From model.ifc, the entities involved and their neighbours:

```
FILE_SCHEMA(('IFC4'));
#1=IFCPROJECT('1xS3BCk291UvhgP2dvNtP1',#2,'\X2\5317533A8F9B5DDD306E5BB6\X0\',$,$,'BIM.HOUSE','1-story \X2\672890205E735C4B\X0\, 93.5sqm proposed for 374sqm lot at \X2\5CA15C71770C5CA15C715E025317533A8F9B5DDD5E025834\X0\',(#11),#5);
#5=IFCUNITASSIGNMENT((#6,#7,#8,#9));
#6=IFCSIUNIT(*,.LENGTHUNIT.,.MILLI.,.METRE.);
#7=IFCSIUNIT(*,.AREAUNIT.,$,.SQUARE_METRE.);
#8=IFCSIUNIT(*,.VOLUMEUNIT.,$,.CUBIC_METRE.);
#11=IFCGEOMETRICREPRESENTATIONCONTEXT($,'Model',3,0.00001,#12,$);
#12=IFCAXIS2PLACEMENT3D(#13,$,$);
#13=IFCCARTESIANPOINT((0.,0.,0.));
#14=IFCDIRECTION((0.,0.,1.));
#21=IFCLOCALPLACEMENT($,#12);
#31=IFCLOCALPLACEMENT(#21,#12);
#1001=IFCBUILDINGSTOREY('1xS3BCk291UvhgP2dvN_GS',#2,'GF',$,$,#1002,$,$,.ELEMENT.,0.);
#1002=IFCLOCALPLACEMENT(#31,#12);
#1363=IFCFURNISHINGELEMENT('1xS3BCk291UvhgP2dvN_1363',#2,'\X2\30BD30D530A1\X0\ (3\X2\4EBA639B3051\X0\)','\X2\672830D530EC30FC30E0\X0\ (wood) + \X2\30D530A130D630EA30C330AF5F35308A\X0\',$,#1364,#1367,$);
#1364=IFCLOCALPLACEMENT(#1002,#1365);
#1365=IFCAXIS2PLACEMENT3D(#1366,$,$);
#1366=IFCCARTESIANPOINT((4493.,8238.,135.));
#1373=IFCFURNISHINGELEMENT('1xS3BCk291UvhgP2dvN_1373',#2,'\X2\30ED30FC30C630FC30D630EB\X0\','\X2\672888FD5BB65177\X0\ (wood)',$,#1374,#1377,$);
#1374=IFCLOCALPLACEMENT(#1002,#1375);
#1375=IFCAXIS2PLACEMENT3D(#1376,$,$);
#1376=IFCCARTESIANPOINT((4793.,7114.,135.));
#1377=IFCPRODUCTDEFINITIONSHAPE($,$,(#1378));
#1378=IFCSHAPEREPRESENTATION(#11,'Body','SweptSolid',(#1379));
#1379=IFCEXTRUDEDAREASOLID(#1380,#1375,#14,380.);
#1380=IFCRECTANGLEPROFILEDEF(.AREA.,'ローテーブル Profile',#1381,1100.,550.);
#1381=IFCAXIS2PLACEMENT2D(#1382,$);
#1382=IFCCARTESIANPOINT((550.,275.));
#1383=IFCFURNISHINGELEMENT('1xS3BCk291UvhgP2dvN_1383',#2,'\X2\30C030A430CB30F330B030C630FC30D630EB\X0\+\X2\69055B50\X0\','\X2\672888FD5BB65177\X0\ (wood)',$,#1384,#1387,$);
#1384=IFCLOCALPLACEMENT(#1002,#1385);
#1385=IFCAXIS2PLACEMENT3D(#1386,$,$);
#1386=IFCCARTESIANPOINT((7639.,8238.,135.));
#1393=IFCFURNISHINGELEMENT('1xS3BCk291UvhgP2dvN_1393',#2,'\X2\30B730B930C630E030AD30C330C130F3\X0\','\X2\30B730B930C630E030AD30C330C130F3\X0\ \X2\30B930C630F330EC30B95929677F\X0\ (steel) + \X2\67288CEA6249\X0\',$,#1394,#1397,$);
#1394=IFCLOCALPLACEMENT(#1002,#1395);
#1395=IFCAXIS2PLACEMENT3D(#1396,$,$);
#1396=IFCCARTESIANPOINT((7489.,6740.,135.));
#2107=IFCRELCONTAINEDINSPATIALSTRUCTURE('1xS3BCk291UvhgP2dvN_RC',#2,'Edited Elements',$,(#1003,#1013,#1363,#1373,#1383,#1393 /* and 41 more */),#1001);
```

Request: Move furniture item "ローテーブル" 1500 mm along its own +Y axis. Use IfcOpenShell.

```python
import ifcopenshell
import ifcopenshell.api.geometry
import ifcopenshell.util.placement

model = ifcopenshell.open("model.ifc")

item = model.by_guid("1xS3BCk291UvhgP2dvN_1373")
matrix = ifcopenshell.util.placement.get_local_placement(item.ObjectPlacement)
matrix[:3, 3] += matrix[:3, 1] * 1500.0
ifcopenshell.api.geometry.edit_object_placement(model, product=item, matrix=matrix, is_si=False)

print(ifcopenshell.util.placement.get_local_placement(item.ObjectPlacement).round(3) + 0.0)

model.write("model_edited.ifc")
```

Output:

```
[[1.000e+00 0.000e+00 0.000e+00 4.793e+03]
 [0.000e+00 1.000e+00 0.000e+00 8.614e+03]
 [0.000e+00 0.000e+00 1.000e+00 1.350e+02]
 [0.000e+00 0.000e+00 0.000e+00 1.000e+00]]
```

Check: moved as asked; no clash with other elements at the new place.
